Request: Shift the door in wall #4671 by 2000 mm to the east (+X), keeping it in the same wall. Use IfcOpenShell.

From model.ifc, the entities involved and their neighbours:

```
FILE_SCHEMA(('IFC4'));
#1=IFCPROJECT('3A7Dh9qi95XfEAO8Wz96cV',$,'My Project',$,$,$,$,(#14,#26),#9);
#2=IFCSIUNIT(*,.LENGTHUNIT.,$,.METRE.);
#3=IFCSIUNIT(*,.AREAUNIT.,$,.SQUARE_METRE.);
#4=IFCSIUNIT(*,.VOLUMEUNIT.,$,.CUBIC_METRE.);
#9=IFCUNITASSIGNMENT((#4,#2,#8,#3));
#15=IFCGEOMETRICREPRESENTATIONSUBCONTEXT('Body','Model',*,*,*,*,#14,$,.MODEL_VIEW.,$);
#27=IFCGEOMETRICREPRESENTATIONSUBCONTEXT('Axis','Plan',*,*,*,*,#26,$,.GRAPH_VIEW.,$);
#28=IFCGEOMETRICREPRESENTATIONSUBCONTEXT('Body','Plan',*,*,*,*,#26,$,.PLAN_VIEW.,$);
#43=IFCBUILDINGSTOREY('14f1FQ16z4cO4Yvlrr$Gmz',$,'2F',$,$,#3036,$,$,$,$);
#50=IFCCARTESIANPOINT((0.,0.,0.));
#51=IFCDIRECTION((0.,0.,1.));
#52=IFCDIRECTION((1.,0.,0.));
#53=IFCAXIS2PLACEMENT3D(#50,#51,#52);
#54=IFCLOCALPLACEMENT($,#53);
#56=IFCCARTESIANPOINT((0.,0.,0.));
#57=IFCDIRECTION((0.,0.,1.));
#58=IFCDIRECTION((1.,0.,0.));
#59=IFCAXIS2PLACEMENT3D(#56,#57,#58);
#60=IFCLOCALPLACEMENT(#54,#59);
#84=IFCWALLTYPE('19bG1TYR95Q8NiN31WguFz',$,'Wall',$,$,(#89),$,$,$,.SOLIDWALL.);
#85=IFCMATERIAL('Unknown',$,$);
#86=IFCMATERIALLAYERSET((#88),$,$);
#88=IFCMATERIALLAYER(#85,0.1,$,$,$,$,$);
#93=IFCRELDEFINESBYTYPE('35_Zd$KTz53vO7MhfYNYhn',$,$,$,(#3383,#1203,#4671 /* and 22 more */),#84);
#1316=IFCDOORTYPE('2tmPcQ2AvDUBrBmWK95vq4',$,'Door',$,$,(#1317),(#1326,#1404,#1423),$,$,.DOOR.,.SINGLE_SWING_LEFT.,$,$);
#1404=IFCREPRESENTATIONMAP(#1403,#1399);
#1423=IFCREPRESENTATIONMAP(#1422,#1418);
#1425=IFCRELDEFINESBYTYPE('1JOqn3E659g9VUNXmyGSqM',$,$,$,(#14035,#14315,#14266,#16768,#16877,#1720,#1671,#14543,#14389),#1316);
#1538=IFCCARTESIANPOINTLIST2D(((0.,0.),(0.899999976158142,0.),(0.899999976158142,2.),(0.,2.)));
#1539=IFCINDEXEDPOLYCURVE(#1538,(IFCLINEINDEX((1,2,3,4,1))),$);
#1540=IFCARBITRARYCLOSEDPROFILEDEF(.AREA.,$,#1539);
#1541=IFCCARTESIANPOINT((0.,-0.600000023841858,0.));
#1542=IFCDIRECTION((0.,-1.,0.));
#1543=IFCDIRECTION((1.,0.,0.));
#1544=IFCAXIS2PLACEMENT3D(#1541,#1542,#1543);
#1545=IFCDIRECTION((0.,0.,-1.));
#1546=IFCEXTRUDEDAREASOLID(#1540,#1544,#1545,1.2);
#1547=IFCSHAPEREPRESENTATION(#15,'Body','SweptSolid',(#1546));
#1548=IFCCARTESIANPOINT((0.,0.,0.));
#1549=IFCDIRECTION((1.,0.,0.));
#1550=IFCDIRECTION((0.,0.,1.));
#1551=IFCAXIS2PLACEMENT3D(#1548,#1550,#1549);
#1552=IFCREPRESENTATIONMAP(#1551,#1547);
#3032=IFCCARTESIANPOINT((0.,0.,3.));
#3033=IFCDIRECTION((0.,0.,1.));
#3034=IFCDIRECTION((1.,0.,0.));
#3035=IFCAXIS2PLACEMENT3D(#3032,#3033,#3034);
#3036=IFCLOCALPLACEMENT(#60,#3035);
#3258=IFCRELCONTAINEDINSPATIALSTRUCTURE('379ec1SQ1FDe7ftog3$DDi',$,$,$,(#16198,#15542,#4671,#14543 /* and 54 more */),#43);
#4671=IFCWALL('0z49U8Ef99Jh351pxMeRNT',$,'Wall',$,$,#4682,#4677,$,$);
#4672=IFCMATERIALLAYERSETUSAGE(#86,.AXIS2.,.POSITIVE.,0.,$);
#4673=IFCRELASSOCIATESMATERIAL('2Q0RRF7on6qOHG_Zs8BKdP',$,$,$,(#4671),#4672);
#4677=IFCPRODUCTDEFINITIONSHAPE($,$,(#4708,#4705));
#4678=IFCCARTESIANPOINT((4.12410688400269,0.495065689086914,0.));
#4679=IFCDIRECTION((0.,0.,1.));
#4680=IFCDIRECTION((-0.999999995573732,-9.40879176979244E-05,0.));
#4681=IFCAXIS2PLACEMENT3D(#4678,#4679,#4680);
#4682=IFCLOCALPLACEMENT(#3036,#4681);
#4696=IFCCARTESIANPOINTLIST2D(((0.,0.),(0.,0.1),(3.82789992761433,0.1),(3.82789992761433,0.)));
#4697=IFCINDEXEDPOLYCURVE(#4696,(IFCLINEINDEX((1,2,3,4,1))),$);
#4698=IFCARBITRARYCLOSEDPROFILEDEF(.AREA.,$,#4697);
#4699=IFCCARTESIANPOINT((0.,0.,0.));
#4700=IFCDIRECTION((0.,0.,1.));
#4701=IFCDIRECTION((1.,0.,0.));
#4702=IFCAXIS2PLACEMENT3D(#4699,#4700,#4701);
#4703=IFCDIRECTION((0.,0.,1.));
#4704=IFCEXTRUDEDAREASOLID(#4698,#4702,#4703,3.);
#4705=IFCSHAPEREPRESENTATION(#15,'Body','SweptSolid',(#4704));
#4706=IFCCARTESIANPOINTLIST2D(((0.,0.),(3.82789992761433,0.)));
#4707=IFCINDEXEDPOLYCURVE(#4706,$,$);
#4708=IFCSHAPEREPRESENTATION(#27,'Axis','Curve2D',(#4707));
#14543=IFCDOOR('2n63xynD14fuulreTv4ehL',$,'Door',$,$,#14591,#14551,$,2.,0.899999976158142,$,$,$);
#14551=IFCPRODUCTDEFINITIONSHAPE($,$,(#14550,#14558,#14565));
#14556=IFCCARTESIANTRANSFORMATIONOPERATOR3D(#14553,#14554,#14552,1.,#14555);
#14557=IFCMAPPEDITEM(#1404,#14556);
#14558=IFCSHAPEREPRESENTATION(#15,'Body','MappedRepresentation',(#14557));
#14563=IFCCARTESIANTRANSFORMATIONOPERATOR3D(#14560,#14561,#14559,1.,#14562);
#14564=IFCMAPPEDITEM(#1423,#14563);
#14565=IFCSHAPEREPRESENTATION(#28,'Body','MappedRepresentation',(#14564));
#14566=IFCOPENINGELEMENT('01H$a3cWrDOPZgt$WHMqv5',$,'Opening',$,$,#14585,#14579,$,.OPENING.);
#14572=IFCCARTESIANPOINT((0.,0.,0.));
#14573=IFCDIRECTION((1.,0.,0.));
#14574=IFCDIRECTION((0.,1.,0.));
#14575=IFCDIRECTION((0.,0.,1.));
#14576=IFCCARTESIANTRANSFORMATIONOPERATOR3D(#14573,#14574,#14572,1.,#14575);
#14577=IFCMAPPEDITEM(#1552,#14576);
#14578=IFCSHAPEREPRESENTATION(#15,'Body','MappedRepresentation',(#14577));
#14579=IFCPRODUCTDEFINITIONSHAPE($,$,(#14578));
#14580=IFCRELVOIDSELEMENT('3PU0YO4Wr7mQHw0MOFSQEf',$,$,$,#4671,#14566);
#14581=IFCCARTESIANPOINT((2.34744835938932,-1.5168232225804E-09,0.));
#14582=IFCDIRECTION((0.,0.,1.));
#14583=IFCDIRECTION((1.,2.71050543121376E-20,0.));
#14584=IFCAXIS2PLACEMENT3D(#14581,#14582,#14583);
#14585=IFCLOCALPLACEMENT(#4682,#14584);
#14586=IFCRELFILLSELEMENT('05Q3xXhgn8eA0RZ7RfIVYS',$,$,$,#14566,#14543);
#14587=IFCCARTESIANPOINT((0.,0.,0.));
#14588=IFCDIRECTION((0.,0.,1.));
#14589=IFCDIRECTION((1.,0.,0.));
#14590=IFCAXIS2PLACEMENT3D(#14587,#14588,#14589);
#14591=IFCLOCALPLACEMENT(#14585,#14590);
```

```python
import ifcopenshell
import ifcopenshell.api.geometry
import ifcopenshell.util.placement

model = ifcopenshell.open("model.ifc")

door = model.by_guid("2n63xynD14fuulreTv4ehL")
opening = door.FillsVoids[0].RelatingOpeningElement
wall = opening.VoidsElements[0].RelatingBuildingElement

wall_matrix = ifcopenshell.util.placement.get_local_placement(wall.ObjectPlacement)
shift = wall_matrix[:3, 0] * -2.0
before = ifcopenshell.util.placement.get_local_placement(door.ObjectPlacement)[:3, 3].copy()

# The door is placed relative to its opening, so it follows when the opening moves.
matrix = ifcopenshell.util.placement.get_local_placement(opening.ObjectPlacement)
matrix[:3, 3] += shift
ifcopenshell.api.geometry.edit_object_placement(
    model, product=opening, matrix=matrix, is_si=False, should_transform_children=True
)

after = ifcopenshell.util.placement.get_local_placement(door.ObjectPlacement)[:3, 3]
print("door moved by", (after - before).round(3) + 0.0)

model.write("model_updated.ifc")
```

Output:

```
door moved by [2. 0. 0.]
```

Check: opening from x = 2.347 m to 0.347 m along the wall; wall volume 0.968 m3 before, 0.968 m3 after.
